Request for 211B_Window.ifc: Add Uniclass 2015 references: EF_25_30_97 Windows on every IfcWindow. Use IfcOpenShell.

First a look at what the model holds.

```python
import ifcopenshell

model = ifcopenshell.open("211B_Window.ifc")
print(model.schema)
print("classifications:", [c.Name for c in model.by_type("IfcClassification")])
for ifc_class in ("IfcDoor", "IfcRoof", "IfcStair", "IfcWall", "IfcWindow"):
    print(ifc_class, len(model.by_type(ifc_class)))
```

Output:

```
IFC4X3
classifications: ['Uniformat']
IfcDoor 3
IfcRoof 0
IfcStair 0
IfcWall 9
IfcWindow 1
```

```python
import ifcopenshell
import ifcopenshell.api.classification

model = ifcopenshell.open("211B_Window.ifc")

system = ifcopenshell.api.classification.add_classification(model, classification="Uniclass 2015")

codes = {
    "IfcWindow": ("EF_25_30_97", "Windows"),
}
for ifc_class, (code, name) in codes.items():
    products = model.by_type(ifc_class)
    ifcopenshell.api.classification.add_reference(
        model, products=products, classification=system, identification=code, name=name
    )
    print(code, len(products))

model.write("211B_Window-out.ifc")
```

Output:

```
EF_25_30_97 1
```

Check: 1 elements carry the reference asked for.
